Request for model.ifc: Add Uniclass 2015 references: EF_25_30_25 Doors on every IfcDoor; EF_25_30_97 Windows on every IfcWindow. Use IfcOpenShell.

First a look at what the model holds.

```python
import ifcopenshell

model = ifcopenshell.open("model.ifc")
print(model.schema)
print("classifications:", [c.Name for c in model.by_type("IfcClassification")])
for ifc_class in ("IfcDoor", "IfcRoof", "IfcStair", "IfcWall", "IfcWindow"):
    print(ifc_class, len(model.by_type(ifc_class)))
```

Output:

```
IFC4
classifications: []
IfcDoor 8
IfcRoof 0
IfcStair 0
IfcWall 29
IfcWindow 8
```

```python
import ifcopenshell
import ifcopenshell.api.classification

model = ifcopenshell.open("model.ifc")

system = ifcopenshell.api.classification.add_classification(model, classification="Uniclass 2015")

codes = {
    "IfcDoor": ("EF_25_30_25", "Doors"),
    "IfcWindow": ("EF_25_30_97", "Windows"),
}
for ifc_class, (code, name) in codes.items():
    products = model.by_type(ifc_class)
    ifcopenshell.api.classification.add_reference(
        model, products=products, classification=system, identification=code, name=name
    )
    print(code, len(products))

model.write("model-out.ifc")
```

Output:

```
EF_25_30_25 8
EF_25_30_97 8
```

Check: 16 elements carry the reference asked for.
